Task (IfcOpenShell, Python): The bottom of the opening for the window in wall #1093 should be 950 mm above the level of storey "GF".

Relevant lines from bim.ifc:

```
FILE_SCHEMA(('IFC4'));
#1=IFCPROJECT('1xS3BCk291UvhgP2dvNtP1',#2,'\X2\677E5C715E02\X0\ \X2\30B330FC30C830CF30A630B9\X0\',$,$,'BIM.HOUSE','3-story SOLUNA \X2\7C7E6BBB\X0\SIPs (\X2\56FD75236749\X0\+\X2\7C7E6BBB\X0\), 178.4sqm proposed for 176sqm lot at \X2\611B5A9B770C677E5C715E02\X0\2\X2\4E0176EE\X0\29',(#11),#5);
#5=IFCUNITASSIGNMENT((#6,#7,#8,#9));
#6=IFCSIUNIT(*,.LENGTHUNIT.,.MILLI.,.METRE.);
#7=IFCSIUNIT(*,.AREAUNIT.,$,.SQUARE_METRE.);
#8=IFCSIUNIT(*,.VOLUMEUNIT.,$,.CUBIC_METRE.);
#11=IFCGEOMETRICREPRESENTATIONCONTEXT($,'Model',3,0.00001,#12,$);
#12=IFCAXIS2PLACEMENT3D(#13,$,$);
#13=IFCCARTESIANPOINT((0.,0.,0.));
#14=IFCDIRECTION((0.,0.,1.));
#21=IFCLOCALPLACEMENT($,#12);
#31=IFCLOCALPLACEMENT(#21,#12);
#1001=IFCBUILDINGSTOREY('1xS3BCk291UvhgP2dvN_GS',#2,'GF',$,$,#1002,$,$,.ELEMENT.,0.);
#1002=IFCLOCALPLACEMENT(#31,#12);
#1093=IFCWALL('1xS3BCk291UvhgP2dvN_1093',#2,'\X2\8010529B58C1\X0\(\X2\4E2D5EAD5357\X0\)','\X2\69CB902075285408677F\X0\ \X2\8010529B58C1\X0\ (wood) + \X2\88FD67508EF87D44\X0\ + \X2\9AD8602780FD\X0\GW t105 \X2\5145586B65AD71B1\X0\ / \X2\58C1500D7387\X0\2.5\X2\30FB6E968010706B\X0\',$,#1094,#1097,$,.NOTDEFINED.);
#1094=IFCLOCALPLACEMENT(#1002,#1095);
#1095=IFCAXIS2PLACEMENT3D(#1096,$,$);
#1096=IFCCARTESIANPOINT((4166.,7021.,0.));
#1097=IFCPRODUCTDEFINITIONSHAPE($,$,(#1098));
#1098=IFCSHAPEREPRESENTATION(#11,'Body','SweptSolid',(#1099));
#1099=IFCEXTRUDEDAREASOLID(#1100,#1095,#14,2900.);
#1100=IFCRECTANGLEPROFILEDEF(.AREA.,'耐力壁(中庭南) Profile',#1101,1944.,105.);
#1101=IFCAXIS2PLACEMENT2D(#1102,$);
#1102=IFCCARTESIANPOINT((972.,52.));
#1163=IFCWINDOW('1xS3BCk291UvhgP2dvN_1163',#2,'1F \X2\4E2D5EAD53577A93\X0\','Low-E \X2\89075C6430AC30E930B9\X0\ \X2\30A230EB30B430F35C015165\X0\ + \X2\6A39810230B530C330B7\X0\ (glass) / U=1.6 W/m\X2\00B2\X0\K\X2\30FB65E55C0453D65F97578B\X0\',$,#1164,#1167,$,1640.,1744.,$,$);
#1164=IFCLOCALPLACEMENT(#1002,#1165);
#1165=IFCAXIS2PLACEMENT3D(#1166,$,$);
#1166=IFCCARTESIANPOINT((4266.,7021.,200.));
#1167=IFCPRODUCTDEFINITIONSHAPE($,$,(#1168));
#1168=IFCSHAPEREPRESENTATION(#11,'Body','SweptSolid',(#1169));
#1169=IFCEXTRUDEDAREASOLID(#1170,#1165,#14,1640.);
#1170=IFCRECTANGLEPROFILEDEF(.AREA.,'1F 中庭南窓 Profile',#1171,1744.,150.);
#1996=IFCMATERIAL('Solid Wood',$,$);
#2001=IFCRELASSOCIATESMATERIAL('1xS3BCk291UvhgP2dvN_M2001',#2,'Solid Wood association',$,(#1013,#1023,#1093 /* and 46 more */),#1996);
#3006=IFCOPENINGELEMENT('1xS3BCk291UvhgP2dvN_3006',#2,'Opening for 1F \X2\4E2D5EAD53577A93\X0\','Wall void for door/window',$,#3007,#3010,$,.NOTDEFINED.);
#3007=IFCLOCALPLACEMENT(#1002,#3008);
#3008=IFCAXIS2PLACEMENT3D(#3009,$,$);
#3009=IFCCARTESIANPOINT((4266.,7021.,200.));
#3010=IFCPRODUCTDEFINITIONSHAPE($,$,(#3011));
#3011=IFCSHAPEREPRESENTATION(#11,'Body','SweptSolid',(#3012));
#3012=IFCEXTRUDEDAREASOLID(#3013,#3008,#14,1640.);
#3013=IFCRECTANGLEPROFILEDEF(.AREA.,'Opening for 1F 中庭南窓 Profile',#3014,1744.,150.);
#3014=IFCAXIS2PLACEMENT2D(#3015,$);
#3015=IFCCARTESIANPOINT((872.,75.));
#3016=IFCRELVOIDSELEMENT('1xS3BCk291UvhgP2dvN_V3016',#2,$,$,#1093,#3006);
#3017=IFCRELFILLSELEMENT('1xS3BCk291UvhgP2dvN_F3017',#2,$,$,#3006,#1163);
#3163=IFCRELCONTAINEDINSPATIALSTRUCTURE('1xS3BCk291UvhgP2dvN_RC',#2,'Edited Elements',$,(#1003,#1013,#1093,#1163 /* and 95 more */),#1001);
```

```python
import numpy as np
import ifcopenshell
import ifcopenshell.api.geometry
import ifcopenshell.geom
import ifcopenshell.util.element
import ifcopenshell.util.placement
import ifcopenshell.util.shape
import ifcopenshell.util.unit

model = ifcopenshell.open("bim.ifc")
unit_scale = ifcopenshell.util.unit.calculate_unit_scale(model)

window = model.by_guid("1xS3BCk291UvhgP2dvN_1163")
opening = window.FillsVoids[0].RelatingOpeningElement
storey = ifcopenshell.util.element.get_container(window, ifc_class="IfcBuildingStorey")
level = ifcopenshell.util.placement.get_local_placement(storey.ObjectPlacement)[2, 3]

# The opening's origin need not be at the sill, so measure its lowest point.
shape = ifcopenshell.geom.create_shape(ifcopenshell.geom.settings(), opening)
bottom = ifcopenshell.util.shape.get_shape_bottom_elevation(shape, shape.geometry) / unit_scale
dz = level + 0.95 / unit_scale - bottom

shift = np.array([0.0, 0.0, dz])
# The window is not placed relative to its opening, so move both.
for product in (opening, window):
    matrix = ifcopenshell.util.placement.get_local_placement(product.ObjectPlacement)
    matrix[:3, 3] += shift
    ifcopenshell.api.geometry.edit_object_placement(model, product=product, matrix=matrix, is_si=False)

print(f"moved by {dz * unit_scale:+.3f} m")

model.write("bim_updated.ifc")
```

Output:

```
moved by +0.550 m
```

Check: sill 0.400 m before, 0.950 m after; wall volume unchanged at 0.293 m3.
